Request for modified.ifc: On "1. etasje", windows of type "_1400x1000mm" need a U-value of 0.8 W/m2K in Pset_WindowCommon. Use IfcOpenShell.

First a look at what the model holds.

```python
import ifcopenshell
import ifcopenshell.util.element

model = ifcopenshell.open("modified.ifc")
print(model.schema)
storey = next(s for s in model.by_type("IfcBuildingStorey") if s.Name == "1. etasje")
windows = [e for e in ifcopenshell.util.element.get_decomposition(storey) if e.is_a("IfcWindow")]
seen = {}
for e in windows:
    element_type = ifcopenshell.util.element.get_type(e)
    key = (element_type.Name if element_type != e and element_type else None, ifcopenshell.util.element.get_pset(e, "Pset_WindowCommon", "ThermalTransmittance"))
    seen[key] = seen.get(key, 0) + 1
for (name, value), count in sorted(seen.items(), key=str):
    print(count, "x", name, "|", value)
```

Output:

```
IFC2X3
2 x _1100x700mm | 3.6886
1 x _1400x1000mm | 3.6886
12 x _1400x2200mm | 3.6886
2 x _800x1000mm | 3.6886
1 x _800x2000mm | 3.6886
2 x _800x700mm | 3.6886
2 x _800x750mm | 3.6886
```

```python
import ifcopenshell
import ifcopenshell.api.pset
import ifcopenshell.util.element

model = ifcopenshell.open("modified.ifc")

storey = next(s for s in model.by_type("IfcBuildingStorey") if s.Name == "1. etasje")
windows = [e for e in ifcopenshell.util.element.get_decomposition(storey) if e.is_a("IfcWindow")]

count = 0
for e in windows:
    element_type = ifcopenshell.util.element.get_type(e)
    if element_type in (None, e) or element_type.Name != "_1400x1000mm":
        continue
    # add_pset returns the element's existing set when there is one.
    pset = ifcopenshell.api.pset.add_pset(model, product=e, name="Pset_WindowCommon")
    ifcopenshell.api.pset.edit_pset(model, pset=pset, properties={"ThermalTransmittance": 0.8})
    count += 1

print(count, "windows updated")

model.write("modified_edited.ifc")
```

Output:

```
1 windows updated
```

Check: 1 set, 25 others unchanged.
